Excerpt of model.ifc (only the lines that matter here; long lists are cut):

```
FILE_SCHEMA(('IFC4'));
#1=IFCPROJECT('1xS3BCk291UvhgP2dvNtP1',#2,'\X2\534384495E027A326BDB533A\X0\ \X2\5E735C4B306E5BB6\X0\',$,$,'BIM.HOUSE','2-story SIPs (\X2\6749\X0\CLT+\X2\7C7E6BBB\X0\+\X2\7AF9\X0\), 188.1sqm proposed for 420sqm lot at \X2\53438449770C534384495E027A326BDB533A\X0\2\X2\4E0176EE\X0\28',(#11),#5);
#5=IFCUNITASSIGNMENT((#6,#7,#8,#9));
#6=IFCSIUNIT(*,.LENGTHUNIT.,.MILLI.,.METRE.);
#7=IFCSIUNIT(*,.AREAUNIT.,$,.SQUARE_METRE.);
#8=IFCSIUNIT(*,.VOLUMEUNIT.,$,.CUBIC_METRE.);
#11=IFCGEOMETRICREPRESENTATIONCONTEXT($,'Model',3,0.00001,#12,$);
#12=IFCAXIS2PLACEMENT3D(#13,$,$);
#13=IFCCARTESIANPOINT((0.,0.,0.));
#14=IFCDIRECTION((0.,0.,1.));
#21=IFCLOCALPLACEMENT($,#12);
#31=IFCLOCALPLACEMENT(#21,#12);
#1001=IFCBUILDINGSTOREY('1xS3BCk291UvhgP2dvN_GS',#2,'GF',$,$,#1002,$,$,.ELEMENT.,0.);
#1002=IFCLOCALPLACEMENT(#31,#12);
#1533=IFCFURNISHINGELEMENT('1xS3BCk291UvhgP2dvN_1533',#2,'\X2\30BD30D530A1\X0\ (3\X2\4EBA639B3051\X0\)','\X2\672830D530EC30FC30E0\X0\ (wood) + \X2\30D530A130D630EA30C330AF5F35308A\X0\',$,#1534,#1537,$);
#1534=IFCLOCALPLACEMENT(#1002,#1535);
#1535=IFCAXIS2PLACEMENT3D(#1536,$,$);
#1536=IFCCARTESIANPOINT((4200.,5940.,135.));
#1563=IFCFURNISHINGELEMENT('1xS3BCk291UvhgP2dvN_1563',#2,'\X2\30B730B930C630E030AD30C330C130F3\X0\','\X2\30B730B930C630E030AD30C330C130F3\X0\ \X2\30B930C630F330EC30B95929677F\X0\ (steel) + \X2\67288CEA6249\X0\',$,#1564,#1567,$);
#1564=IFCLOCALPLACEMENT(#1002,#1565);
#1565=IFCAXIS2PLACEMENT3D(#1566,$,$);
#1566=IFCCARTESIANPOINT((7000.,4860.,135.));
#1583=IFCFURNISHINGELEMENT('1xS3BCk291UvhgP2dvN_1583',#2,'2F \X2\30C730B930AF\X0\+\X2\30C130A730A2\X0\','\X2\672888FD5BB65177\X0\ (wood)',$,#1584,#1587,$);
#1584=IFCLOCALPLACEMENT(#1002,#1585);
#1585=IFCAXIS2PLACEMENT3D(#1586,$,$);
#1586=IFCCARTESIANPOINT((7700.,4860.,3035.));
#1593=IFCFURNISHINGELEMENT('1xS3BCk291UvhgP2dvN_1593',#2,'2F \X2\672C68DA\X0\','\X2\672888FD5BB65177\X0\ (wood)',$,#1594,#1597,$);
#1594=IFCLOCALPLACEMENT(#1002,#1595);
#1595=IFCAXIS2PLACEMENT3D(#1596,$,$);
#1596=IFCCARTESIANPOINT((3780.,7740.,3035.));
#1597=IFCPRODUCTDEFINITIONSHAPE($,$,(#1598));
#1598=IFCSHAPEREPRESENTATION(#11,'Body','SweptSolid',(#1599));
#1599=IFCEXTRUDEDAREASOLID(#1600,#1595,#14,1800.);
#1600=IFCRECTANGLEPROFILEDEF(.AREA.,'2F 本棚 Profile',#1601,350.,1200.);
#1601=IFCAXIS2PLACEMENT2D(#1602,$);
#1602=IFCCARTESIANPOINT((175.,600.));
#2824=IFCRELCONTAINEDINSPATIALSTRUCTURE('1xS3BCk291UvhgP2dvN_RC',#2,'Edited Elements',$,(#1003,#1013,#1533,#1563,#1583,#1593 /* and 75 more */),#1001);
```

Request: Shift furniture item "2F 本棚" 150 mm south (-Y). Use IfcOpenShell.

```python
import ifcopenshell
import ifcopenshell.api.geometry
import ifcopenshell.util.placement
import ifcopenshell.util.unit

model = ifcopenshell.open("model.ifc")
unit_scale = ifcopenshell.util.unit.calculate_unit_scale(model)

item = model.by_id(1593)
matrix = ifcopenshell.util.placement.get_local_placement(item.ObjectPlacement)
matrix[1, 3] -= 0.15 / unit_scale
ifcopenshell.api.geometry.edit_object_placement(model, product=item, matrix=matrix, is_si=False)

print(ifcopenshell.util.placement.get_local_placement(item.ObjectPlacement).round(3) + 0.0)

model.write("model_updated.ifc")
```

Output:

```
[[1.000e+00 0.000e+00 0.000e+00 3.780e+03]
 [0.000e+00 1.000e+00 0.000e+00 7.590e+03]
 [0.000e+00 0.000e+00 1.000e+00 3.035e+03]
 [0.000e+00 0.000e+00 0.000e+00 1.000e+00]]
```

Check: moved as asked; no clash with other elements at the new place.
